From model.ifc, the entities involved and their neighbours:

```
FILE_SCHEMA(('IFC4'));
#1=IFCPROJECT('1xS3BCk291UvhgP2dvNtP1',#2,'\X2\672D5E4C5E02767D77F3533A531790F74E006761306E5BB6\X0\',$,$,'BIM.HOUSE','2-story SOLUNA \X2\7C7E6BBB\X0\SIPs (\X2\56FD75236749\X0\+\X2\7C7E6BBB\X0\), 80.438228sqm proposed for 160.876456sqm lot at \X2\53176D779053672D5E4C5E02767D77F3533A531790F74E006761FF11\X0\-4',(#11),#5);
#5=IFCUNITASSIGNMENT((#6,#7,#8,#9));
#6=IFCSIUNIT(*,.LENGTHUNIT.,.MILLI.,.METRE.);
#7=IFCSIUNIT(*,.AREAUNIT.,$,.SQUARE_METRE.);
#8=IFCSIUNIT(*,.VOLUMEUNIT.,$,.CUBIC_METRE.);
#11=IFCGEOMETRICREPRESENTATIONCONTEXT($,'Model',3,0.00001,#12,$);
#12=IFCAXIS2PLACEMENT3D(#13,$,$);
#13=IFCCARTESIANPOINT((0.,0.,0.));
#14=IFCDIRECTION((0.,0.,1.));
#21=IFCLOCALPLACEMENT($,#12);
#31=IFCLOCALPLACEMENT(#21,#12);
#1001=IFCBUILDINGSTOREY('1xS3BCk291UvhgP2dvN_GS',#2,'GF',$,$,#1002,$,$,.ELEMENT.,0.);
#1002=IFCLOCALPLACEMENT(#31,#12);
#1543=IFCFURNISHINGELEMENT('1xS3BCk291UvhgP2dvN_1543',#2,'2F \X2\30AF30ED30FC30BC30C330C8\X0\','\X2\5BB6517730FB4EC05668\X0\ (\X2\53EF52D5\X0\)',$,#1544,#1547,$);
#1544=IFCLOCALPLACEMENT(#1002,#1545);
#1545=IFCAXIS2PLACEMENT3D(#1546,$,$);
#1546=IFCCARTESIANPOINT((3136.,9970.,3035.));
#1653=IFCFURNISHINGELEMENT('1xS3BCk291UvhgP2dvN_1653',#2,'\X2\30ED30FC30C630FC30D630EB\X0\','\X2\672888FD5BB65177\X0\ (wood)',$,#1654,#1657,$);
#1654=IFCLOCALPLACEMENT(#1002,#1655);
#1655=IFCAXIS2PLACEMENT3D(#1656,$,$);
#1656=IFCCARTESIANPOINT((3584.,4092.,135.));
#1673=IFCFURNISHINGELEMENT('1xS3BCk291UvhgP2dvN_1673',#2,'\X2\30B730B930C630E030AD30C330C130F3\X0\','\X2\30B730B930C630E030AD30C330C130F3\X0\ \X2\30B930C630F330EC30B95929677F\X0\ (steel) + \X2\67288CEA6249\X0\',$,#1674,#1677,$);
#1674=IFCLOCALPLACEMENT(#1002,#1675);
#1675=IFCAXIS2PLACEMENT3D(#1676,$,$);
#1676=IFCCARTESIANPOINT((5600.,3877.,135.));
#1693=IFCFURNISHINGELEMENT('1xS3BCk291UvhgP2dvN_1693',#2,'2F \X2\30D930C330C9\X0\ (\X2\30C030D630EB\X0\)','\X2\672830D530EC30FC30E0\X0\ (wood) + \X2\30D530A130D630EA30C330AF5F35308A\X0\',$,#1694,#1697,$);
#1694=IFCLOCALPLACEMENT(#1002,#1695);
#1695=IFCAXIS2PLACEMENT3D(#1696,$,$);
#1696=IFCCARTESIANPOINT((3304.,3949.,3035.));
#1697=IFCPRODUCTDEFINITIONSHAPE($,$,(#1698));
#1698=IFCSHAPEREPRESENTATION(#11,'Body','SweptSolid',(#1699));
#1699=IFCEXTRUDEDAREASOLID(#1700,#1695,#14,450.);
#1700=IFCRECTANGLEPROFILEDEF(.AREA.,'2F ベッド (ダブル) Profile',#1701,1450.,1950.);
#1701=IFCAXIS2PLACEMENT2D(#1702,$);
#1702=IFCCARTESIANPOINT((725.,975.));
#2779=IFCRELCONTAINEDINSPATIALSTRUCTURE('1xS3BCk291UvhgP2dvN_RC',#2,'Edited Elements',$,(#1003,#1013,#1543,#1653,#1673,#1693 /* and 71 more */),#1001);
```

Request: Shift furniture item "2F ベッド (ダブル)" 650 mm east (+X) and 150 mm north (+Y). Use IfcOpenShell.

```python
import ifcopenshell
import ifcopenshell.api.geometry
import ifcopenshell.util.placement
import ifcopenshell.util.unit

model = ifcopenshell.open("model.ifc")
unit_scale = ifcopenshell.util.unit.calculate_unit_scale(model)

item = model.by_guid("1xS3BCk291UvhgP2dvN_1693")
matrix = ifcopenshell.util.placement.get_local_placement(item.ObjectPlacement)
matrix[0, 3] += 0.65 / unit_scale
matrix[1, 3] += 0.15 / unit_scale
ifcopenshell.api.geometry.edit_object_placement(model, product=item, matrix=matrix, is_si=False)

print(ifcopenshell.util.placement.get_local_placement(item.ObjectPlacement).round(3) + 0.0)

model.write("model_rev.ifc")
```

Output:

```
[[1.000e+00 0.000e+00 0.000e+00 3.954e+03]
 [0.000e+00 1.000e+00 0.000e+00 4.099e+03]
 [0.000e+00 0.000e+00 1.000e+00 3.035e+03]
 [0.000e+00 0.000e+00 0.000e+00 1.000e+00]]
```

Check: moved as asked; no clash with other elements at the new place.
